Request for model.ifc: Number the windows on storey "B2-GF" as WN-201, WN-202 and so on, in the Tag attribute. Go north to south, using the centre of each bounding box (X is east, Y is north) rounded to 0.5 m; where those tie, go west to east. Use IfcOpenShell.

First a look at what the model holds.

```python
import ifcopenshell
import ifcopenshell.util.element
import ifcopenshell.util.placement

model = ifcopenshell.open("model.ifc")
print(model.schema)
storey = next(s for s in model.by_type("IfcBuildingStorey") if s.Name == "B2-GF")
windows = [e for e in ifcopenshell.util.element.get_decomposition(storey) if e.is_a("IfcWindow")]
for e in sorted(windows, key=lambda e: e.id()):
    origin = ifcopenshell.util.placement.get_local_placement(e.ObjectPlacement)[:3, 3]
    print(e.id(), e.Tag, e.Name, origin.round(2) + 0.0, sep=" | ")
```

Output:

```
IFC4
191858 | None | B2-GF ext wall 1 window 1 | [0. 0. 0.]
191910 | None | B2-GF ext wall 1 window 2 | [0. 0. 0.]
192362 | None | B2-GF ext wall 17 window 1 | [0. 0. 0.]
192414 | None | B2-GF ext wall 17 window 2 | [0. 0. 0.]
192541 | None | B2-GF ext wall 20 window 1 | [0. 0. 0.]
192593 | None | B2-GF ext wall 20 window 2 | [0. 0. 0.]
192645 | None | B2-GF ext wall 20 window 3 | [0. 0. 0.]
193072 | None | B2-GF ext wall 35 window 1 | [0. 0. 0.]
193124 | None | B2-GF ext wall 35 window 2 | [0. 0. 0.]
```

```python
import ifcopenshell
import ifcopenshell.geom
import ifcopenshell.util.element
import ifcopenshell.util.shape

model = ifcopenshell.open("model.ifc")
settings = ifcopenshell.geom.settings()
settings.set("use-world-coords", True)


def centre(element):
    shape = ifcopenshell.geom.create_shape(settings, element)
    return ifcopenshell.util.shape.get_bbox_centroid(shape.geometry)


storey = next(s for s in model.by_type("IfcBuildingStorey") if s.Name == "B2-GF")
windows = [e for e in ifcopenshell.util.element.get_decomposition(storey) if e.is_a("IfcWindow")]

# Insertion points can sit at a corner or the storey origin, so sort by the geometry (in metres).
centres = {e: centre(e) for e in windows}
windows.sort(key=lambda e: (-round(centres[e][1] / 0.5), centres[e][0]))

for i, e in enumerate(windows, start=1):
    number = f"WN-2{i:02d}"
    e.Tag = number
    print(e.id(), number)

model.write("model_edited.ifc")
```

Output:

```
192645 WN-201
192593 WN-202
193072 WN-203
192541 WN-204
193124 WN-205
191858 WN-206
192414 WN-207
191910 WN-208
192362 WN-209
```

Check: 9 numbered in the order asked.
